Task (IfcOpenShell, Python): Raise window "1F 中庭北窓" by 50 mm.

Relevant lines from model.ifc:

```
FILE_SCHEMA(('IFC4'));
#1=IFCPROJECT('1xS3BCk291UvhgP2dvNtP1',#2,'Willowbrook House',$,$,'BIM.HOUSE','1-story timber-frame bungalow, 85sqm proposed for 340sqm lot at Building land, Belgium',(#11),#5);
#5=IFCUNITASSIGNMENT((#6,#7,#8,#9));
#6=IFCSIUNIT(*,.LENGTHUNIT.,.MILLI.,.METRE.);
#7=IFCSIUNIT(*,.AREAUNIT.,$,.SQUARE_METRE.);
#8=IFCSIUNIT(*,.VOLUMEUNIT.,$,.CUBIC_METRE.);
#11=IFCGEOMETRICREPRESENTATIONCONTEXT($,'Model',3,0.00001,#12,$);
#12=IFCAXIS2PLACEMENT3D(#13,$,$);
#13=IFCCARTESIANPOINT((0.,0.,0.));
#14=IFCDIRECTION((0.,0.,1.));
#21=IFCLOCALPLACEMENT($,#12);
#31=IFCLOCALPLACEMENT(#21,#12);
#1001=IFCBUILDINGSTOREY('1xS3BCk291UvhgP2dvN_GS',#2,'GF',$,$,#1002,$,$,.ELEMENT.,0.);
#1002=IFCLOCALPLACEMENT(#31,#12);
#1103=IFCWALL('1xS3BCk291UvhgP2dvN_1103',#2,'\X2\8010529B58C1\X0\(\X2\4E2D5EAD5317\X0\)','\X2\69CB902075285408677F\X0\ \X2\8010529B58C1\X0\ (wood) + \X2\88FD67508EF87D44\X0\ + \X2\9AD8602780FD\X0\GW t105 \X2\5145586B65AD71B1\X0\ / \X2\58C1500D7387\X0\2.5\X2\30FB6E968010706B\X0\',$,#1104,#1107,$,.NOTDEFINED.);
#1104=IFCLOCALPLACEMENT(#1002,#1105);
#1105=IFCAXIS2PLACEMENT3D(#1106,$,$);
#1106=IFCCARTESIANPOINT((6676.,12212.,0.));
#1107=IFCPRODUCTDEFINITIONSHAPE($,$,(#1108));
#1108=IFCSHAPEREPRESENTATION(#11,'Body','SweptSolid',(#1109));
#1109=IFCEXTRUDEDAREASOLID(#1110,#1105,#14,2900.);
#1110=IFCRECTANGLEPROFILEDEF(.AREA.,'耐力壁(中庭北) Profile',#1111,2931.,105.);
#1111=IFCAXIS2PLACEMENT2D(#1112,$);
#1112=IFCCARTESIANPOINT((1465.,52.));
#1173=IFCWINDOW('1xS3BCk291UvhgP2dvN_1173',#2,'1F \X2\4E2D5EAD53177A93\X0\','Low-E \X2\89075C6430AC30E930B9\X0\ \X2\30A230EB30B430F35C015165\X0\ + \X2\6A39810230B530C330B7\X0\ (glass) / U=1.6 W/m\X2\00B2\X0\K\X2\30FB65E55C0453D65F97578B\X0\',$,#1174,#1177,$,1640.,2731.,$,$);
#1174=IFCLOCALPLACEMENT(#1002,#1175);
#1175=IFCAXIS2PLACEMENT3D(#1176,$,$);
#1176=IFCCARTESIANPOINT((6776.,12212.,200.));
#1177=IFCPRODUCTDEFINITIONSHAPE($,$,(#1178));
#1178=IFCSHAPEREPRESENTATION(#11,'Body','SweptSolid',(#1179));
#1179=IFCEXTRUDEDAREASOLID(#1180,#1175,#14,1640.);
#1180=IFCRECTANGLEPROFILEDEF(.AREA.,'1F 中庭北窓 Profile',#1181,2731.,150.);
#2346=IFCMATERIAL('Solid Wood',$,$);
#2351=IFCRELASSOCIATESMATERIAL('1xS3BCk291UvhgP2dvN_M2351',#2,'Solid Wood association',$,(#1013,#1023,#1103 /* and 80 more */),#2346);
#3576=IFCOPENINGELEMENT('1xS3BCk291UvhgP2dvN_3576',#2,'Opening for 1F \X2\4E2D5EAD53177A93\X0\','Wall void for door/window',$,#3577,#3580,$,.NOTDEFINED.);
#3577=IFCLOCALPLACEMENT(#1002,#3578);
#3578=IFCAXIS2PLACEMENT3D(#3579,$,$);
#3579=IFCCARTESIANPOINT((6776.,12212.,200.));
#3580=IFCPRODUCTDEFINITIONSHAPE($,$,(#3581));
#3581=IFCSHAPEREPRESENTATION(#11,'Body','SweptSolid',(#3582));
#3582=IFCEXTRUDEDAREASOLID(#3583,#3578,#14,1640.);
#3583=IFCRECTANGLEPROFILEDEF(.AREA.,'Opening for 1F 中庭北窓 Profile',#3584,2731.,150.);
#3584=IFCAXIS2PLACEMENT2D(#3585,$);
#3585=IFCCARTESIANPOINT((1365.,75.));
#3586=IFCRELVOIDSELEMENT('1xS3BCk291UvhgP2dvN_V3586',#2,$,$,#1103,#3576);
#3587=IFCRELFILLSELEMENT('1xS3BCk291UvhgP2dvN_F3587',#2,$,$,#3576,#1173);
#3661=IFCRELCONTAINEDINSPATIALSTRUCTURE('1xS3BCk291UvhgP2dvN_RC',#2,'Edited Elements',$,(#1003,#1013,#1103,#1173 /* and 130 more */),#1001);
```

```python
import numpy as np
import ifcopenshell
import ifcopenshell.api.geometry
import ifcopenshell.util.placement
import ifcopenshell.util.unit

model = ifcopenshell.open("model.ifc")
unit_scale = ifcopenshell.util.unit.calculate_unit_scale(model)

window = model.by_id(1173)
opening = window.FillsVoids[0].RelatingOpeningElement
dz = 50.0

shift = np.array([0.0, 0.0, dz])
# The window is not placed relative to its opening, so move both.
for product in (opening, window):
    matrix = ifcopenshell.util.placement.get_local_placement(product.ObjectPlacement)
    matrix[:3, 3] += shift
    ifcopenshell.api.geometry.edit_object_placement(model, product=product, matrix=matrix, is_si=False)

print(f"moved by {dz * unit_scale:+.3f} m")

model.write("model_updated.ifc")
```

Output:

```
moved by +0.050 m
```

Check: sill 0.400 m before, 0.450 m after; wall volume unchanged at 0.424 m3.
